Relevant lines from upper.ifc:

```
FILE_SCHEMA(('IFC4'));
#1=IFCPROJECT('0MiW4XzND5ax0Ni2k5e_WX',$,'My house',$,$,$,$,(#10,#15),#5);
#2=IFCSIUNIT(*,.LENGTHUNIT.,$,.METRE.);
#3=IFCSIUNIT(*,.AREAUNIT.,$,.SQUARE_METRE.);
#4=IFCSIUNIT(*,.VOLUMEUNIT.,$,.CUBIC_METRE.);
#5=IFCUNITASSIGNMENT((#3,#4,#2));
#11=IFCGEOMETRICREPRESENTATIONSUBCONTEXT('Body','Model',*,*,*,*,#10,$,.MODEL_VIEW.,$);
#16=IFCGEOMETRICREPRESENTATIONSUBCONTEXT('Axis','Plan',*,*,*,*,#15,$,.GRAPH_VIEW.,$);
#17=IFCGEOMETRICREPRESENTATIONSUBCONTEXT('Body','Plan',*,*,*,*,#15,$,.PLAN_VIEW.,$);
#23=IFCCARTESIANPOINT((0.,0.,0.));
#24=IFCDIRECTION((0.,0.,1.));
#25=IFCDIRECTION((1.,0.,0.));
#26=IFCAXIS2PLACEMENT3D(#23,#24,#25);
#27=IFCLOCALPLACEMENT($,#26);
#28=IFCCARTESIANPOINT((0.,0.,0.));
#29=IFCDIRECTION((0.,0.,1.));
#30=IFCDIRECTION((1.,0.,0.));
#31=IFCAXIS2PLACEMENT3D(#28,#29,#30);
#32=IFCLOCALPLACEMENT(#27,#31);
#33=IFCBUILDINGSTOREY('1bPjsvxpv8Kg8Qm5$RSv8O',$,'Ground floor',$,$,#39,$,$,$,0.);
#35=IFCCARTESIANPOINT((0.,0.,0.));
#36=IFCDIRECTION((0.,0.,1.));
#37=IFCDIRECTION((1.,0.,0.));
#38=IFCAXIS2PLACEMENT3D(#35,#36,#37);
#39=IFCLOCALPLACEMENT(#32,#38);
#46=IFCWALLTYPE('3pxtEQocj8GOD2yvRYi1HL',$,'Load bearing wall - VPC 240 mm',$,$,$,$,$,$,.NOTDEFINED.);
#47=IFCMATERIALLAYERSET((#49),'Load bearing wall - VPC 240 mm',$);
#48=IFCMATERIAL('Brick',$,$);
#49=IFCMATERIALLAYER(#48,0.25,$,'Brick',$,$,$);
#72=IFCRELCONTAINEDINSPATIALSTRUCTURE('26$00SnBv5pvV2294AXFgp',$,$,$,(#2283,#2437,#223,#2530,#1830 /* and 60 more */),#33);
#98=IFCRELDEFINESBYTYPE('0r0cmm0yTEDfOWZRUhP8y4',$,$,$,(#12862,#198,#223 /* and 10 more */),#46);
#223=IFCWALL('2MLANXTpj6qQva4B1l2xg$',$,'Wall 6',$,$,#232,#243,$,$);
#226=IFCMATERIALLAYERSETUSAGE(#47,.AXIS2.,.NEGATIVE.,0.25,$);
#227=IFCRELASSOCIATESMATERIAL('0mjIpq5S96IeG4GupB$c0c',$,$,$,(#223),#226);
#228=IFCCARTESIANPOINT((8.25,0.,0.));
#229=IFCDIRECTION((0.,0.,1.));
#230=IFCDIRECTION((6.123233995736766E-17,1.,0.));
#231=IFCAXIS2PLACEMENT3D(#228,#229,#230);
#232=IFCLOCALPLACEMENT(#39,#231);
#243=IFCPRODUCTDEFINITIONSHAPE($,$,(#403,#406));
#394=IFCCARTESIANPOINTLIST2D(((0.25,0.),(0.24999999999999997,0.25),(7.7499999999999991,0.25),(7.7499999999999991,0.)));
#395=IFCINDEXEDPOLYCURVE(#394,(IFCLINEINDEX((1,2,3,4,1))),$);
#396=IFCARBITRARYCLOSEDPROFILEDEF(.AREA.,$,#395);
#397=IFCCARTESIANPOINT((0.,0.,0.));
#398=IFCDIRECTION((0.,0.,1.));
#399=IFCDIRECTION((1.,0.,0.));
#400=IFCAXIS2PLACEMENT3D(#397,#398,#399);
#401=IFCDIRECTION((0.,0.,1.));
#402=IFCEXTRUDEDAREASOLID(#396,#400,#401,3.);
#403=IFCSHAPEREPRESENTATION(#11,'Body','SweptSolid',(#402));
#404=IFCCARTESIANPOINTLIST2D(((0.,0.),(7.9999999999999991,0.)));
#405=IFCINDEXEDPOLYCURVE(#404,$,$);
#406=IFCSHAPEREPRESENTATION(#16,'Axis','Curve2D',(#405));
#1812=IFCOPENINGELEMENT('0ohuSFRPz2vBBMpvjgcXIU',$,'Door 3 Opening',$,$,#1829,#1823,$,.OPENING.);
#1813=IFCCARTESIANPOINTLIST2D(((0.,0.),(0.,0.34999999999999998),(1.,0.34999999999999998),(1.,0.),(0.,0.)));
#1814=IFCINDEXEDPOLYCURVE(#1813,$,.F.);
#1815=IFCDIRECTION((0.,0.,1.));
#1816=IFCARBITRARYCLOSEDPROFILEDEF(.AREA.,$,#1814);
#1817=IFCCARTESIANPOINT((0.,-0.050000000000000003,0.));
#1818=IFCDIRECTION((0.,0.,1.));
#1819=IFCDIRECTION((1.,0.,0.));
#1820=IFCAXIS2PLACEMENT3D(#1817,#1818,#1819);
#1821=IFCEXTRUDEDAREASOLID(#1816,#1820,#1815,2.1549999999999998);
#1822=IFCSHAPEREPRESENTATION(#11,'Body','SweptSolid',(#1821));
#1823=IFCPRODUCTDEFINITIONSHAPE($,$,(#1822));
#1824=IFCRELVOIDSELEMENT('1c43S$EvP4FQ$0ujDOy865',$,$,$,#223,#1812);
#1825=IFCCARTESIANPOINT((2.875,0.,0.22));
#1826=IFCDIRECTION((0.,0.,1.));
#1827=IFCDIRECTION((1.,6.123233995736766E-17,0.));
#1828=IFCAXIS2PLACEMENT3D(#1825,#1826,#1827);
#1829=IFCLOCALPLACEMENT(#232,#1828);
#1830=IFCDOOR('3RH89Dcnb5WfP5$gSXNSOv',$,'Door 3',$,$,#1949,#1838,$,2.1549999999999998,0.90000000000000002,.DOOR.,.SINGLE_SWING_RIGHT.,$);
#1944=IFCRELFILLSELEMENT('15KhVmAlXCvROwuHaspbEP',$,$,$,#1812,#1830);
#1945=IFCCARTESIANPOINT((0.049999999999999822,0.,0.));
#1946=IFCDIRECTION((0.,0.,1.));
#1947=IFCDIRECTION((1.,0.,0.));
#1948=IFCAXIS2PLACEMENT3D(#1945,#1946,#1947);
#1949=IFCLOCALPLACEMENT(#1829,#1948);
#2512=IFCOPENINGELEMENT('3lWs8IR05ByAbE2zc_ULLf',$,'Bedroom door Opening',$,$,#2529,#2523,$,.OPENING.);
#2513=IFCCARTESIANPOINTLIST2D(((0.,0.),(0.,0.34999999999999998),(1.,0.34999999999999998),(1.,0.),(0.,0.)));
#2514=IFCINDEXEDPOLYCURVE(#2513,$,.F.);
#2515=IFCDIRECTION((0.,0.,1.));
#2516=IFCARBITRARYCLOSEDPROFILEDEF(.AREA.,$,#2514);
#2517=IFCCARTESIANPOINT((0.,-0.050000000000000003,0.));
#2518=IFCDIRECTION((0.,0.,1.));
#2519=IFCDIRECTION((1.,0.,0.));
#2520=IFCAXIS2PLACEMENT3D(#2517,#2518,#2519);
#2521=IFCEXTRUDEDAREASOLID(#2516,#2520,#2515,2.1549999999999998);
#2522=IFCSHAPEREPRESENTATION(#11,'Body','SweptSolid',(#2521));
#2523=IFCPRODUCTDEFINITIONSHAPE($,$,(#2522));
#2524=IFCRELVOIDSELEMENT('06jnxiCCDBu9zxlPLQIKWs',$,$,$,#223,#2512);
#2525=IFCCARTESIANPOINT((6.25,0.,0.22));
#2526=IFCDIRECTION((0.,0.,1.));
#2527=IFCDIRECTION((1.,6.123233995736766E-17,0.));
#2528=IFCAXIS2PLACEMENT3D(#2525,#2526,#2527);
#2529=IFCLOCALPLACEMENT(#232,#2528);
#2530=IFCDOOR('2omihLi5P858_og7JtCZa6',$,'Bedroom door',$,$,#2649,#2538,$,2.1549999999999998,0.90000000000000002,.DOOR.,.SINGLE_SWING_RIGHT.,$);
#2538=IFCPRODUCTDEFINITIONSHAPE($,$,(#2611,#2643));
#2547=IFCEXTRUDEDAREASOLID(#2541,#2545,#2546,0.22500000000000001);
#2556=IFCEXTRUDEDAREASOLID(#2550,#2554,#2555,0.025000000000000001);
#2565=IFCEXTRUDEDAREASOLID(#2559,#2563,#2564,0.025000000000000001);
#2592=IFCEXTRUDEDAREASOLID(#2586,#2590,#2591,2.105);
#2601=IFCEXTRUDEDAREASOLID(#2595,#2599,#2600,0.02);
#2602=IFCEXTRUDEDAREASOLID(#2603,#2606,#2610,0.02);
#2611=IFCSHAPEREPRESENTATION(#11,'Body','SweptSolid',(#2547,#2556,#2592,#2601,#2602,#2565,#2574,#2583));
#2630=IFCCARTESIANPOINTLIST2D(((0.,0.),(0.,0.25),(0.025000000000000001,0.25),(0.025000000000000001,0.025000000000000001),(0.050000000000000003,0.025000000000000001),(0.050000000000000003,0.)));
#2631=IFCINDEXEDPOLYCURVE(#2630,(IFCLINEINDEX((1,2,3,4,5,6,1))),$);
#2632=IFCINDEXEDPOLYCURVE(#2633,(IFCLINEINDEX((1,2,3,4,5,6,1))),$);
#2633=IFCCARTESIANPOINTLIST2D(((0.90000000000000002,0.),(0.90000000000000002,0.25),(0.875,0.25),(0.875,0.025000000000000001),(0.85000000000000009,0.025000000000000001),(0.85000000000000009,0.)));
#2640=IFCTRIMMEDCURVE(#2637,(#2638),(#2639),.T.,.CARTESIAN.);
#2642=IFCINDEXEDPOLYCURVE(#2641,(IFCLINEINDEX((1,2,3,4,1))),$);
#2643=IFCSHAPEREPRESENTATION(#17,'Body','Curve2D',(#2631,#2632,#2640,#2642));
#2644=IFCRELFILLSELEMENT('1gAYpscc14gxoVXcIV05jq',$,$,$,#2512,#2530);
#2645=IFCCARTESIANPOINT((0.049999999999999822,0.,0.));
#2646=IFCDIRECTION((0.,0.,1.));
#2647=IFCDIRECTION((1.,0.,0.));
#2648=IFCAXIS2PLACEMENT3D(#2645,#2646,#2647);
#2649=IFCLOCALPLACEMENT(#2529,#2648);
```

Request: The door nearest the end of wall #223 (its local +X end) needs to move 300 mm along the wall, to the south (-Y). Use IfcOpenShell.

```python
import ifcopenshell
import ifcopenshell.api.geometry
import ifcopenshell.util.placement

model = ifcopenshell.open("upper.ifc")

door = model.by_guid("2omihLi5P858_og7JtCZa6")
opening = door.FillsVoids[0].RelatingOpeningElement
wall = opening.VoidsElements[0].RelatingBuildingElement

wall_matrix = ifcopenshell.util.placement.get_local_placement(wall.ObjectPlacement)
shift = wall_matrix[:3, 0] * -0.3
before = ifcopenshell.util.placement.get_local_placement(door.ObjectPlacement)[:3, 3].copy()

# The door is placed relative to its opening, so it follows when the opening moves.
matrix = ifcopenshell.util.placement.get_local_placement(opening.ObjectPlacement)
matrix[:3, 3] += shift
ifcopenshell.api.geometry.edit_object_placement(
    model, product=opening, matrix=matrix, is_si=False, should_transform_children=True
)

after = ifcopenshell.util.placement.get_local_placement(door.ObjectPlacement)[:3, 3]
print("door moved by", (after - before).round(3) + 0.0)

model.write("upper_v2.ifc")
```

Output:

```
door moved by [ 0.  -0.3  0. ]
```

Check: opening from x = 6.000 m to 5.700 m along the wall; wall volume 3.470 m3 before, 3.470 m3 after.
